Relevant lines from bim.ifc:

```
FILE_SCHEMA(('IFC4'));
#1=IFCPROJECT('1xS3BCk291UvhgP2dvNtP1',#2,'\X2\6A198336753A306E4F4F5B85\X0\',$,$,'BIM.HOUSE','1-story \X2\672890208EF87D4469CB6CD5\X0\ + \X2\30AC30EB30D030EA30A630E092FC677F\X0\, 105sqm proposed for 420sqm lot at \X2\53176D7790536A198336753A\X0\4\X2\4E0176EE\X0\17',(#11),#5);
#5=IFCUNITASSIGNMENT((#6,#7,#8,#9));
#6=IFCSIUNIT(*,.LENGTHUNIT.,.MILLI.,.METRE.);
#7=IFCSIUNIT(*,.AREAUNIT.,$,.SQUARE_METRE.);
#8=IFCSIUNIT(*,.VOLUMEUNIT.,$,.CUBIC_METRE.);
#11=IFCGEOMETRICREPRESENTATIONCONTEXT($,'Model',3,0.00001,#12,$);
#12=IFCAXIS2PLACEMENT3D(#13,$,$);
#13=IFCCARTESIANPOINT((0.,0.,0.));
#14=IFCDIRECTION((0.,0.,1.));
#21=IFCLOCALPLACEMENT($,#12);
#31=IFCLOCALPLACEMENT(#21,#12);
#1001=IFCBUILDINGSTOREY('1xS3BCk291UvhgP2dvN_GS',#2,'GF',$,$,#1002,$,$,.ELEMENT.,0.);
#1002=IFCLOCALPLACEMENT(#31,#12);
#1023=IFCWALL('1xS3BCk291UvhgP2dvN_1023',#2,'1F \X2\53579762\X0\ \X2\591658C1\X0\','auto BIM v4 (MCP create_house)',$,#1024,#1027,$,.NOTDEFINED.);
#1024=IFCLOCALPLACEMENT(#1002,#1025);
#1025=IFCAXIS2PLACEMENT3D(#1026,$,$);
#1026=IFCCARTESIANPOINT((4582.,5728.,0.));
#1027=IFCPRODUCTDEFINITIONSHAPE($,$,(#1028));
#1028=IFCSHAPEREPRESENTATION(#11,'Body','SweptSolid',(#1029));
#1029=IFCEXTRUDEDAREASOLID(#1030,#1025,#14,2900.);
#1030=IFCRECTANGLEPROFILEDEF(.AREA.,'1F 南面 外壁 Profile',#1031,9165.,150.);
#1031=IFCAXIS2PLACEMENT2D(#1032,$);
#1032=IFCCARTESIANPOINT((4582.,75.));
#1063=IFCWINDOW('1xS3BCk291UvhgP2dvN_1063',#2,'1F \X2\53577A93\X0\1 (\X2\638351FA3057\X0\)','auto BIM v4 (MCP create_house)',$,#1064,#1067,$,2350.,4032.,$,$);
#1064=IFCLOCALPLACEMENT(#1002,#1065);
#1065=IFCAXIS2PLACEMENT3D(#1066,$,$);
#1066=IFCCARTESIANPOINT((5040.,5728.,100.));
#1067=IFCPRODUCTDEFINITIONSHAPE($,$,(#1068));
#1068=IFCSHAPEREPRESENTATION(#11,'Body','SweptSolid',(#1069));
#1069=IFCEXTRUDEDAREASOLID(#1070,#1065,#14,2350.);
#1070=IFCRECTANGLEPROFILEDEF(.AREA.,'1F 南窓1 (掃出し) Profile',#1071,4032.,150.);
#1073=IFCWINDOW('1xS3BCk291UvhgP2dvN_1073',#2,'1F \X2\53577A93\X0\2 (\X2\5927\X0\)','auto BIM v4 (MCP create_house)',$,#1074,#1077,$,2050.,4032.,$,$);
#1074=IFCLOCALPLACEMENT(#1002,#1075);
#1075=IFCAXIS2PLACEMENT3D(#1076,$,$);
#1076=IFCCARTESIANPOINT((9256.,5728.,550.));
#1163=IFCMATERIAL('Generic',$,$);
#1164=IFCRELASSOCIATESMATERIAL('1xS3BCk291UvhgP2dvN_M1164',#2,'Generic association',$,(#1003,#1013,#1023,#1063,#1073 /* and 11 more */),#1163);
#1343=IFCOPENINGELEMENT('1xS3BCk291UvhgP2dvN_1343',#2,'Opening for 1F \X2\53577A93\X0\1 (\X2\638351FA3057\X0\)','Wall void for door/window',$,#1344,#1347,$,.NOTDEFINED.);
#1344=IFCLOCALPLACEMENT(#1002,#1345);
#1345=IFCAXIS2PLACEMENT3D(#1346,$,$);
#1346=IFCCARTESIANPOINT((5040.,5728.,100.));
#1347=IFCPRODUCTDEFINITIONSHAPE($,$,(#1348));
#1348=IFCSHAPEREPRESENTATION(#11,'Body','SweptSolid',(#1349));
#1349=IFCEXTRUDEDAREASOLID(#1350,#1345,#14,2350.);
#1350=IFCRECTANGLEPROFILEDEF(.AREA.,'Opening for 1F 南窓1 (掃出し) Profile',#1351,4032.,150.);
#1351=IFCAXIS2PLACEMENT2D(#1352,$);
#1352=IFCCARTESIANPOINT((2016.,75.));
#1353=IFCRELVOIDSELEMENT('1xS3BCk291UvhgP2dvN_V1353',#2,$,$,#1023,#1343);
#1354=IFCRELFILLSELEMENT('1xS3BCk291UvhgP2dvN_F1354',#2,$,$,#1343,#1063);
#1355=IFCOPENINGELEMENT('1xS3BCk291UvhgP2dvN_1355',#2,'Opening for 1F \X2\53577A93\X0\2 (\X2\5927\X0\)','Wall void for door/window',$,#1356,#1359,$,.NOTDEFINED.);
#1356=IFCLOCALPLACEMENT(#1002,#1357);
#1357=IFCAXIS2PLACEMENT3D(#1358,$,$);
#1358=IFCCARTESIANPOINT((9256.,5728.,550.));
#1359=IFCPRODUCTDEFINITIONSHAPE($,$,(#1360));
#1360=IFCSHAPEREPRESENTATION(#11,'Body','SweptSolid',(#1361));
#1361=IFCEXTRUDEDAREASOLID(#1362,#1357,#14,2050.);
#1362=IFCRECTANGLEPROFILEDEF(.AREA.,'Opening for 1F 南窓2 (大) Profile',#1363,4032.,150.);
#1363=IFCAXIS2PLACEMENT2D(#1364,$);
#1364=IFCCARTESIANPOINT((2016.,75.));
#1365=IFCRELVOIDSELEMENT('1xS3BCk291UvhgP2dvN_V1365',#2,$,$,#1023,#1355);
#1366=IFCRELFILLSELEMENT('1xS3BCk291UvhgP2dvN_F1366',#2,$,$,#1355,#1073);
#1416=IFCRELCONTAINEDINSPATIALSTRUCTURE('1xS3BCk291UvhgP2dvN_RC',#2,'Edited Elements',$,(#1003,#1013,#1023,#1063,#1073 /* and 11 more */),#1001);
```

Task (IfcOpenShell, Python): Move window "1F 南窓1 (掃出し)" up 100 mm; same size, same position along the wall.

```python
import numpy as np
import ifcopenshell
import ifcopenshell.api.geometry
import ifcopenshell.util.placement
import ifcopenshell.util.unit

model = ifcopenshell.open("bim.ifc")
unit_scale = ifcopenshell.util.unit.calculate_unit_scale(model)

window = model.by_guid("1xS3BCk291UvhgP2dvN_1063")
opening = window.FillsVoids[0].RelatingOpeningElement
dz = 0.1 / unit_scale

shift = np.array([0.0, 0.0, dz])
# The window is not placed relative to its opening, so move both.
for product in (opening, window):
    matrix = ifcopenshell.util.placement.get_local_placement(product.ObjectPlacement)
    matrix[:3, 3] += shift
    ifcopenshell.api.geometry.edit_object_placement(model, product=product, matrix=matrix, is_si=False)

print(f"moved by {dz * unit_scale:+.3f} m")

model.write("bim_updated.ifc")
```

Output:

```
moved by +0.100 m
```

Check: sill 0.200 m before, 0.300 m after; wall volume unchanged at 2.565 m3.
